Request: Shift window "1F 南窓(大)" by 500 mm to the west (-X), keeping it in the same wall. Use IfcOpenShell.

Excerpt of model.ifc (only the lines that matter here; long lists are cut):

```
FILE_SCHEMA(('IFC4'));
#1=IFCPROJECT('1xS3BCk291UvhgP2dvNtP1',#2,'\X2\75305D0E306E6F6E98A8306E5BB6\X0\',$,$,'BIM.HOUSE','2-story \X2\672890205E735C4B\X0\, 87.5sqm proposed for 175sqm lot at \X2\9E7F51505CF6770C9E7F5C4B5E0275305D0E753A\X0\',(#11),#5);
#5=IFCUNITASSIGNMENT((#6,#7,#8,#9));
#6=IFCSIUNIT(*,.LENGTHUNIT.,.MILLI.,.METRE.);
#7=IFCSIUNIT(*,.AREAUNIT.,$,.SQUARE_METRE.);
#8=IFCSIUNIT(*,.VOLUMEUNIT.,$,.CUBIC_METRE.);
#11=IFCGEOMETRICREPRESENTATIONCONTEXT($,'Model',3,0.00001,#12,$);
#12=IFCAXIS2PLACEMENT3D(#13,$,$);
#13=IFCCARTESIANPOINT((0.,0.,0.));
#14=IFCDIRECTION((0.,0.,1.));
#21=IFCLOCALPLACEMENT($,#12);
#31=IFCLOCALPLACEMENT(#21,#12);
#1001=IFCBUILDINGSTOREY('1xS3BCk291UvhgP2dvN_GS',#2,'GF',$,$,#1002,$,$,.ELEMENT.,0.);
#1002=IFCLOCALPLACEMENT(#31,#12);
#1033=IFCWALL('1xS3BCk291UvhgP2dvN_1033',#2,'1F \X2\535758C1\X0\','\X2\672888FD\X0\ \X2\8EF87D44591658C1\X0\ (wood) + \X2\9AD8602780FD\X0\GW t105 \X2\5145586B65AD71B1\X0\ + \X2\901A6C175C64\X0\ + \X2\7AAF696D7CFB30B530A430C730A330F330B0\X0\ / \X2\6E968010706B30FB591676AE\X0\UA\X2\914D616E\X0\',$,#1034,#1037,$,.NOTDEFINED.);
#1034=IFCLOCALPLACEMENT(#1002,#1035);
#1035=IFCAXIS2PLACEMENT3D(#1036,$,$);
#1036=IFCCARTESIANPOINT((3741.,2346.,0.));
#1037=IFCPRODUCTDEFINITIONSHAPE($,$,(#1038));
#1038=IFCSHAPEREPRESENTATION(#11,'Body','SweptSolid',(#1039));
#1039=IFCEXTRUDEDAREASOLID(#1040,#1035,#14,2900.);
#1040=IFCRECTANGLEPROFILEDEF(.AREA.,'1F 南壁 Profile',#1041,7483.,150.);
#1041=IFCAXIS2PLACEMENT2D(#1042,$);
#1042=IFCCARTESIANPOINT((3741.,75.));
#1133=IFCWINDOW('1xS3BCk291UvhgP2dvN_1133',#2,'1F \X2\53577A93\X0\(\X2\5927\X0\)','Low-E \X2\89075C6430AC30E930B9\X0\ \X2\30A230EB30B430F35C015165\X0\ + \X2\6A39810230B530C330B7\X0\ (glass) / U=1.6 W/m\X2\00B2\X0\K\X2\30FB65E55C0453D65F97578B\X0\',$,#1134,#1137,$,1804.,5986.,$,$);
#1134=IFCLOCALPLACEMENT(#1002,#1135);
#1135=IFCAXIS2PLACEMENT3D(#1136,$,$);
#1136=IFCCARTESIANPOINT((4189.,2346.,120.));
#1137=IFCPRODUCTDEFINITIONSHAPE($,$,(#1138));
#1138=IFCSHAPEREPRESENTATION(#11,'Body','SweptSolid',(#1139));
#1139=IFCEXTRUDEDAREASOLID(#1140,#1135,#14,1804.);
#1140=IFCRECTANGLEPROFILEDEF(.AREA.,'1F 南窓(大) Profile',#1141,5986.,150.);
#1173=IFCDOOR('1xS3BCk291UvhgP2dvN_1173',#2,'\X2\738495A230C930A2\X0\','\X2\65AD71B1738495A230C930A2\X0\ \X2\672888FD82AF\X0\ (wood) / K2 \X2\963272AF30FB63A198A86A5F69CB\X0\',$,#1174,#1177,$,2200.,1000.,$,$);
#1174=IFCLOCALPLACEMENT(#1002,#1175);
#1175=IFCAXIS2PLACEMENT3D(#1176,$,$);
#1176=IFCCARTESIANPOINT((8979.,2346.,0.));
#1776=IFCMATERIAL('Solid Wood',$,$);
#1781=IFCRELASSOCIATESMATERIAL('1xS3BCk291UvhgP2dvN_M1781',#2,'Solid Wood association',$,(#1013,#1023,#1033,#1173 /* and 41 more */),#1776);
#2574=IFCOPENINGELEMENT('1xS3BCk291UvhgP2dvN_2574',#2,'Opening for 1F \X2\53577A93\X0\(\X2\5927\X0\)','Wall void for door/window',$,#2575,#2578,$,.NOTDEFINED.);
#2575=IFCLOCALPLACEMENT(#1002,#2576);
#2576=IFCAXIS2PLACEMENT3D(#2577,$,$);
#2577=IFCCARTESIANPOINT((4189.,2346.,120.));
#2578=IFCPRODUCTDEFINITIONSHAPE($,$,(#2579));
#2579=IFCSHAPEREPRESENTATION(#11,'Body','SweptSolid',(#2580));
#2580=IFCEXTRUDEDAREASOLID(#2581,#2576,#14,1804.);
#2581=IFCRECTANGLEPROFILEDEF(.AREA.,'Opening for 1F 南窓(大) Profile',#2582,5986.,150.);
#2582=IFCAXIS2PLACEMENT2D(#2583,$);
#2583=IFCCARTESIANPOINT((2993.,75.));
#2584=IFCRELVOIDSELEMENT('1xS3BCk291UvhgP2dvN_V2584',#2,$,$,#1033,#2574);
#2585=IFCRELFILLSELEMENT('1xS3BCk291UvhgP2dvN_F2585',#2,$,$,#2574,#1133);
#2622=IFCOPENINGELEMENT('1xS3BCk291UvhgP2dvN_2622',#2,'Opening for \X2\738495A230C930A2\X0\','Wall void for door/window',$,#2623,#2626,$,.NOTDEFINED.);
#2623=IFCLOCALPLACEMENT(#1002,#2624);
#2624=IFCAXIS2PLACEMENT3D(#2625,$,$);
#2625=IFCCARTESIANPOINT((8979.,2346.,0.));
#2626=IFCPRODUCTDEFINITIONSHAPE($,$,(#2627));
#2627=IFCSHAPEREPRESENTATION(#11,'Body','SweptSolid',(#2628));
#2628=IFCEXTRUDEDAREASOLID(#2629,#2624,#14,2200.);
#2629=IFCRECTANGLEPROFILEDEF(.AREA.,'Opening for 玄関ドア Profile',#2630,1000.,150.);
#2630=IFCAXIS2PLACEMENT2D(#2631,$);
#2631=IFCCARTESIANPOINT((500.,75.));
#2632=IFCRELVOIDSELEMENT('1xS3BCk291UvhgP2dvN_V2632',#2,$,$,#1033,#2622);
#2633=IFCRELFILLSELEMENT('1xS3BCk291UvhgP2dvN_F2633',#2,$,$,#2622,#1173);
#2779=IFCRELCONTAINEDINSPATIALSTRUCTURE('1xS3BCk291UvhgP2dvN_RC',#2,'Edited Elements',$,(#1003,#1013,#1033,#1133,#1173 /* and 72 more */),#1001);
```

```python
import ifcopenshell
import ifcopenshell.api.geometry
import ifcopenshell.util.placement

model = ifcopenshell.open("model.ifc")

window = model.by_guid("1xS3BCk291UvhgP2dvN_1133")
opening = window.FillsVoids[0].RelatingOpeningElement
wall = opening.VoidsElements[0].RelatingBuildingElement

wall_matrix = ifcopenshell.util.placement.get_local_placement(wall.ObjectPlacement)
shift = wall_matrix[:3, 0] * -500.0
before = ifcopenshell.util.placement.get_local_placement(window.ObjectPlacement)[:3, 3].copy()

# The window is not placed relative to its opening, so move both.
for product in (opening, window):
    matrix = ifcopenshell.util.placement.get_local_placement(product.ObjectPlacement)
    matrix[:3, 3] += shift
    ifcopenshell.api.geometry.edit_object_placement(model, product=product, matrix=matrix, is_si=False)

after = ifcopenshell.util.placement.get_local_placement(window.ObjectPlacement)[:3, 3]
print("window moved by", (after - before).round(3) + 0.0)

model.write("model_v2.ifc")
```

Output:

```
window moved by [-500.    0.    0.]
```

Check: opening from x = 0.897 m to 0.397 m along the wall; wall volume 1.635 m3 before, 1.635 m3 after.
